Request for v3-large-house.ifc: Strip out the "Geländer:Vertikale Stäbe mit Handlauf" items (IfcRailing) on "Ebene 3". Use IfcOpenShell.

First a look at what the model holds.

```python
import ifcopenshell
import ifcopenshell.util.element

model = ifcopenshell.open("v3-large-house.ifc")
print(model.schema)
storey = next(s for s in model.by_type("IfcBuildingStorey") if s.Name == "Ebene 3")
railings = [e for e in ifcopenshell.util.element.get_decomposition(storey) if e.is_a("IfcRailing")]
seen = {}
for e in railings:
    element_type = ifcopenshell.util.element.get_type(e)
    name = element_type.Name if element_type not in (None, e) else None
    seen[name] = seen.get(name, 0) + 1
for name, count in sorted(seen.items(), key=str):
    print(count, "x", name)
```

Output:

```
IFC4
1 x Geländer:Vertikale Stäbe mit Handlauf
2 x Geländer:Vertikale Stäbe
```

```python
import ifcopenshell
import ifcopenshell.api.root
import ifcopenshell.util.element

model = ifcopenshell.open("v3-large-house.ifc")

storey = next(s for s in model.by_type("IfcBuildingStorey") if s.Name == "Ebene 3")
railings = [e for e in ifcopenshell.util.element.get_decomposition(storey) if e.is_a("IfcRailing")]
targets = [e for e in railings if (t := ifcopenshell.util.element.get_type(e)) not in (None, e) and t.Name == "Geländer:Vertikale Stäbe mit Handlauf"]

for e in targets:
    ifcopenshell.api.root.remove_product(model, product=e)
print(len(targets), "removed")

model.write("v3-large-house-out.ifc")
```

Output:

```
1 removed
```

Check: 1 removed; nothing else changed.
